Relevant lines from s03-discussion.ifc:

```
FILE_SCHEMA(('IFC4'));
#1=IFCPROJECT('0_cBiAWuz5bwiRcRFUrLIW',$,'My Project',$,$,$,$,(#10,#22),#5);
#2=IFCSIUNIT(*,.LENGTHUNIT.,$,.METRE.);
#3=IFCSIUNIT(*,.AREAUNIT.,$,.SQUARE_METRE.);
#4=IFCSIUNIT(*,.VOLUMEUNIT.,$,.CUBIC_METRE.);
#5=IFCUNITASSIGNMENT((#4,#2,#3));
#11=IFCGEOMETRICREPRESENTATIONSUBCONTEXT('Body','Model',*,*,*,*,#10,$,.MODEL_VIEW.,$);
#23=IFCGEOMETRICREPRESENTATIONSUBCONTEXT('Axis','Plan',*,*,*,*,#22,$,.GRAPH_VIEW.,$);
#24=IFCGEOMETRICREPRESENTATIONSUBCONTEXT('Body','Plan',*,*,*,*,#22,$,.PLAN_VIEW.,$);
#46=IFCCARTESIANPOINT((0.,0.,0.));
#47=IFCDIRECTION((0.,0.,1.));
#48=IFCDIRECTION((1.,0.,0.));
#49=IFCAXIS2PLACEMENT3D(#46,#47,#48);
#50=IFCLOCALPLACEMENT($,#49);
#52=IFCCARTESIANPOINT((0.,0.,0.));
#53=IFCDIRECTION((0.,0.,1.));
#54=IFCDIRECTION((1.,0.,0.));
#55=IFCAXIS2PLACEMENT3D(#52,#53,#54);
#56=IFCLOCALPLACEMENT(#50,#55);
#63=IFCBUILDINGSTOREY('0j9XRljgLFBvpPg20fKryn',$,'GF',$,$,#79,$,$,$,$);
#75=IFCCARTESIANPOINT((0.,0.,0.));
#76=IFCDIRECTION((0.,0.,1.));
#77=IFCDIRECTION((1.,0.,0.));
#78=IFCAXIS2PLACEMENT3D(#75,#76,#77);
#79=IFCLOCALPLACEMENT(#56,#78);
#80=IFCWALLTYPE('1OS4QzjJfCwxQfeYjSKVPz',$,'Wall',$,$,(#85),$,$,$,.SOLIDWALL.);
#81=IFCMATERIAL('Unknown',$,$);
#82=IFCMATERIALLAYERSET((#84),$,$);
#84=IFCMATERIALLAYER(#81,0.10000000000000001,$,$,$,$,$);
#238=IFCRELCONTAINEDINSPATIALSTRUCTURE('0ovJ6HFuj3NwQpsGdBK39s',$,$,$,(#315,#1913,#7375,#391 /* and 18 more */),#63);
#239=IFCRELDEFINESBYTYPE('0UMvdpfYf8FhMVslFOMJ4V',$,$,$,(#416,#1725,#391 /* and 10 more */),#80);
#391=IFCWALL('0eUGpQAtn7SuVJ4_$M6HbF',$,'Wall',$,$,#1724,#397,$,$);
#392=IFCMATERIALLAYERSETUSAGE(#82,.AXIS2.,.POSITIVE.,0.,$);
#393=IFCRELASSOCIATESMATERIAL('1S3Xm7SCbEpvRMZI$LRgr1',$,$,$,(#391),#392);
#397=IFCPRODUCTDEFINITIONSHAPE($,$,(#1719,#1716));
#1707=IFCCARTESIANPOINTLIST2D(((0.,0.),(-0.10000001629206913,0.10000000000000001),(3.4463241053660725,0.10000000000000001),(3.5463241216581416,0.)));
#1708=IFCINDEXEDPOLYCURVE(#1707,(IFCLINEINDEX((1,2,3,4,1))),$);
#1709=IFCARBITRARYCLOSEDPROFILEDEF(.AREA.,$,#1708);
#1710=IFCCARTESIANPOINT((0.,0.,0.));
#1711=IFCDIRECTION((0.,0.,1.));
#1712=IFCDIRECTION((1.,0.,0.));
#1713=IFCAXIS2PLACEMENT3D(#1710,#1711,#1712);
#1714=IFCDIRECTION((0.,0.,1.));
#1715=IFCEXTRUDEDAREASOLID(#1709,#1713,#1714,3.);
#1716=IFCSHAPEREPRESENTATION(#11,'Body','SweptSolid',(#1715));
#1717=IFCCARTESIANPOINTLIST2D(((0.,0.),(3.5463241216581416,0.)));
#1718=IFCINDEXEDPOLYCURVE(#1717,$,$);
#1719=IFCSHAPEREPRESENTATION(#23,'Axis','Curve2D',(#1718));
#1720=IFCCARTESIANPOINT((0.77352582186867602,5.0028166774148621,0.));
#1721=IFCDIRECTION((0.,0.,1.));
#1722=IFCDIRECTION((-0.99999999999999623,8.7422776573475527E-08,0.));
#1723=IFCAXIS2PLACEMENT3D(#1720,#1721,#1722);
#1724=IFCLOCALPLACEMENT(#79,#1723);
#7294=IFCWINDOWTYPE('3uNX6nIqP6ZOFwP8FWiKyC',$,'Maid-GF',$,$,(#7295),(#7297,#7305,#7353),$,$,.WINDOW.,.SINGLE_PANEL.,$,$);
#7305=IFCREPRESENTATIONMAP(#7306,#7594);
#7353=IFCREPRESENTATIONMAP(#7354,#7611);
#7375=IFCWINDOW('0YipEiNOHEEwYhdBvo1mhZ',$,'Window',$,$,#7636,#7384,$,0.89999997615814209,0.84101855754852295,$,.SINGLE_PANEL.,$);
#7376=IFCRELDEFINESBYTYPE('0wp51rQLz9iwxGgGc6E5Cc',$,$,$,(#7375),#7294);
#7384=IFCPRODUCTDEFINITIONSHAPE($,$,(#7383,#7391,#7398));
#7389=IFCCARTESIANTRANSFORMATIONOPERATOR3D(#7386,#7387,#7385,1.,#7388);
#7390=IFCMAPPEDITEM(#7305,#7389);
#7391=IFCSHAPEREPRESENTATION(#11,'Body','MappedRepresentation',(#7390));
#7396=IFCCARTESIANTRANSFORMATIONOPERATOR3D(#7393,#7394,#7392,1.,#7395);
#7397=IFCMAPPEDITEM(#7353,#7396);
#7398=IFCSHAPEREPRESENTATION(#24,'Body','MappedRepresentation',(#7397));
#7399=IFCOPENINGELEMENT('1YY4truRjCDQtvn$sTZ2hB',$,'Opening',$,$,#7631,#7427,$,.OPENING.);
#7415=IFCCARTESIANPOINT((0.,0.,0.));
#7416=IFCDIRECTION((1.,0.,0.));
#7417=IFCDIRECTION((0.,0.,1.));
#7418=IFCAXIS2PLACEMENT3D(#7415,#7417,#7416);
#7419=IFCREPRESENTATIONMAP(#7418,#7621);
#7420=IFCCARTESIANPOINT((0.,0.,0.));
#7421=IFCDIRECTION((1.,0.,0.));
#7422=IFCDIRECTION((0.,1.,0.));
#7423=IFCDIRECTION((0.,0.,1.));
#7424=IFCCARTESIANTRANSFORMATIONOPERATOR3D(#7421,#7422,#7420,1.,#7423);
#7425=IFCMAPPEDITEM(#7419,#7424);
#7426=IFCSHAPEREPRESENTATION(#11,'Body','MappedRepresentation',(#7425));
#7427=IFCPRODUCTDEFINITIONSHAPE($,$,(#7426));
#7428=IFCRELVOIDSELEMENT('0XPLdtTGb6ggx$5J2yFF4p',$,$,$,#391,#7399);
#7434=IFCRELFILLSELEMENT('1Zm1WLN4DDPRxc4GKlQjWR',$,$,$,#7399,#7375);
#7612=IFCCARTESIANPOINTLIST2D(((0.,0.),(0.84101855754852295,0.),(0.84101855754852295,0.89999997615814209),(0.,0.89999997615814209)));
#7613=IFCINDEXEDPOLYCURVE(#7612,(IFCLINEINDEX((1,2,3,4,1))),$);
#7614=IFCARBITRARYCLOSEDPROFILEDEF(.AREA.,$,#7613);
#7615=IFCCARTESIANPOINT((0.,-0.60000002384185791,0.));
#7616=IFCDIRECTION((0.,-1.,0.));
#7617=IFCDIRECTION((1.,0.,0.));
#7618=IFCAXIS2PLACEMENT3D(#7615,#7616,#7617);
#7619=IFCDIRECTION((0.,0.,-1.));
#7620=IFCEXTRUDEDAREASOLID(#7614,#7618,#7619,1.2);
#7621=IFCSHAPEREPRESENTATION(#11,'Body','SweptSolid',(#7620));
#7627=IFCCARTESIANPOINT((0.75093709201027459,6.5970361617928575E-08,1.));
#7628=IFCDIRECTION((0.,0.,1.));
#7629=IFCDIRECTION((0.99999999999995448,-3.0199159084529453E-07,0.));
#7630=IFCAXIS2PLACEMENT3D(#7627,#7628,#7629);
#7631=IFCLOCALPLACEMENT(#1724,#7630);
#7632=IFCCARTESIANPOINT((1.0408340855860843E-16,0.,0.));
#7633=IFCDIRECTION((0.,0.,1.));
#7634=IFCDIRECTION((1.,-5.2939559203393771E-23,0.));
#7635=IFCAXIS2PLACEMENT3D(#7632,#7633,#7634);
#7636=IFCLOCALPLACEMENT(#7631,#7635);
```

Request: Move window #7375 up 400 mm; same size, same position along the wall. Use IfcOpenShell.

```python
import numpy as np
import ifcopenshell
import ifcopenshell.api.geometry
import ifcopenshell.util.placement
import ifcopenshell.util.unit

model = ifcopenshell.open("s03-discussion.ifc")
unit_scale = ifcopenshell.util.unit.calculate_unit_scale(model)

window = model.by_id(7375)
opening = window.FillsVoids[0].RelatingOpeningElement
dz = 0.4 / unit_scale

shift = np.array([0.0, 0.0, dz])
# The window is placed relative to its opening, so it follows when the opening moves.
matrix = ifcopenshell.util.placement.get_local_placement(opening.ObjectPlacement)
matrix[:3, 3] += shift
ifcopenshell.api.geometry.edit_object_placement(
    model, product=opening, matrix=matrix, is_si=False, should_transform_children=True
)

print(f"moved by {dz * unit_scale:+.3f} m")

model.write("s03-discussion_edited.ifc")
```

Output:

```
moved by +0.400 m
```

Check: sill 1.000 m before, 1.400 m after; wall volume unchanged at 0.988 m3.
